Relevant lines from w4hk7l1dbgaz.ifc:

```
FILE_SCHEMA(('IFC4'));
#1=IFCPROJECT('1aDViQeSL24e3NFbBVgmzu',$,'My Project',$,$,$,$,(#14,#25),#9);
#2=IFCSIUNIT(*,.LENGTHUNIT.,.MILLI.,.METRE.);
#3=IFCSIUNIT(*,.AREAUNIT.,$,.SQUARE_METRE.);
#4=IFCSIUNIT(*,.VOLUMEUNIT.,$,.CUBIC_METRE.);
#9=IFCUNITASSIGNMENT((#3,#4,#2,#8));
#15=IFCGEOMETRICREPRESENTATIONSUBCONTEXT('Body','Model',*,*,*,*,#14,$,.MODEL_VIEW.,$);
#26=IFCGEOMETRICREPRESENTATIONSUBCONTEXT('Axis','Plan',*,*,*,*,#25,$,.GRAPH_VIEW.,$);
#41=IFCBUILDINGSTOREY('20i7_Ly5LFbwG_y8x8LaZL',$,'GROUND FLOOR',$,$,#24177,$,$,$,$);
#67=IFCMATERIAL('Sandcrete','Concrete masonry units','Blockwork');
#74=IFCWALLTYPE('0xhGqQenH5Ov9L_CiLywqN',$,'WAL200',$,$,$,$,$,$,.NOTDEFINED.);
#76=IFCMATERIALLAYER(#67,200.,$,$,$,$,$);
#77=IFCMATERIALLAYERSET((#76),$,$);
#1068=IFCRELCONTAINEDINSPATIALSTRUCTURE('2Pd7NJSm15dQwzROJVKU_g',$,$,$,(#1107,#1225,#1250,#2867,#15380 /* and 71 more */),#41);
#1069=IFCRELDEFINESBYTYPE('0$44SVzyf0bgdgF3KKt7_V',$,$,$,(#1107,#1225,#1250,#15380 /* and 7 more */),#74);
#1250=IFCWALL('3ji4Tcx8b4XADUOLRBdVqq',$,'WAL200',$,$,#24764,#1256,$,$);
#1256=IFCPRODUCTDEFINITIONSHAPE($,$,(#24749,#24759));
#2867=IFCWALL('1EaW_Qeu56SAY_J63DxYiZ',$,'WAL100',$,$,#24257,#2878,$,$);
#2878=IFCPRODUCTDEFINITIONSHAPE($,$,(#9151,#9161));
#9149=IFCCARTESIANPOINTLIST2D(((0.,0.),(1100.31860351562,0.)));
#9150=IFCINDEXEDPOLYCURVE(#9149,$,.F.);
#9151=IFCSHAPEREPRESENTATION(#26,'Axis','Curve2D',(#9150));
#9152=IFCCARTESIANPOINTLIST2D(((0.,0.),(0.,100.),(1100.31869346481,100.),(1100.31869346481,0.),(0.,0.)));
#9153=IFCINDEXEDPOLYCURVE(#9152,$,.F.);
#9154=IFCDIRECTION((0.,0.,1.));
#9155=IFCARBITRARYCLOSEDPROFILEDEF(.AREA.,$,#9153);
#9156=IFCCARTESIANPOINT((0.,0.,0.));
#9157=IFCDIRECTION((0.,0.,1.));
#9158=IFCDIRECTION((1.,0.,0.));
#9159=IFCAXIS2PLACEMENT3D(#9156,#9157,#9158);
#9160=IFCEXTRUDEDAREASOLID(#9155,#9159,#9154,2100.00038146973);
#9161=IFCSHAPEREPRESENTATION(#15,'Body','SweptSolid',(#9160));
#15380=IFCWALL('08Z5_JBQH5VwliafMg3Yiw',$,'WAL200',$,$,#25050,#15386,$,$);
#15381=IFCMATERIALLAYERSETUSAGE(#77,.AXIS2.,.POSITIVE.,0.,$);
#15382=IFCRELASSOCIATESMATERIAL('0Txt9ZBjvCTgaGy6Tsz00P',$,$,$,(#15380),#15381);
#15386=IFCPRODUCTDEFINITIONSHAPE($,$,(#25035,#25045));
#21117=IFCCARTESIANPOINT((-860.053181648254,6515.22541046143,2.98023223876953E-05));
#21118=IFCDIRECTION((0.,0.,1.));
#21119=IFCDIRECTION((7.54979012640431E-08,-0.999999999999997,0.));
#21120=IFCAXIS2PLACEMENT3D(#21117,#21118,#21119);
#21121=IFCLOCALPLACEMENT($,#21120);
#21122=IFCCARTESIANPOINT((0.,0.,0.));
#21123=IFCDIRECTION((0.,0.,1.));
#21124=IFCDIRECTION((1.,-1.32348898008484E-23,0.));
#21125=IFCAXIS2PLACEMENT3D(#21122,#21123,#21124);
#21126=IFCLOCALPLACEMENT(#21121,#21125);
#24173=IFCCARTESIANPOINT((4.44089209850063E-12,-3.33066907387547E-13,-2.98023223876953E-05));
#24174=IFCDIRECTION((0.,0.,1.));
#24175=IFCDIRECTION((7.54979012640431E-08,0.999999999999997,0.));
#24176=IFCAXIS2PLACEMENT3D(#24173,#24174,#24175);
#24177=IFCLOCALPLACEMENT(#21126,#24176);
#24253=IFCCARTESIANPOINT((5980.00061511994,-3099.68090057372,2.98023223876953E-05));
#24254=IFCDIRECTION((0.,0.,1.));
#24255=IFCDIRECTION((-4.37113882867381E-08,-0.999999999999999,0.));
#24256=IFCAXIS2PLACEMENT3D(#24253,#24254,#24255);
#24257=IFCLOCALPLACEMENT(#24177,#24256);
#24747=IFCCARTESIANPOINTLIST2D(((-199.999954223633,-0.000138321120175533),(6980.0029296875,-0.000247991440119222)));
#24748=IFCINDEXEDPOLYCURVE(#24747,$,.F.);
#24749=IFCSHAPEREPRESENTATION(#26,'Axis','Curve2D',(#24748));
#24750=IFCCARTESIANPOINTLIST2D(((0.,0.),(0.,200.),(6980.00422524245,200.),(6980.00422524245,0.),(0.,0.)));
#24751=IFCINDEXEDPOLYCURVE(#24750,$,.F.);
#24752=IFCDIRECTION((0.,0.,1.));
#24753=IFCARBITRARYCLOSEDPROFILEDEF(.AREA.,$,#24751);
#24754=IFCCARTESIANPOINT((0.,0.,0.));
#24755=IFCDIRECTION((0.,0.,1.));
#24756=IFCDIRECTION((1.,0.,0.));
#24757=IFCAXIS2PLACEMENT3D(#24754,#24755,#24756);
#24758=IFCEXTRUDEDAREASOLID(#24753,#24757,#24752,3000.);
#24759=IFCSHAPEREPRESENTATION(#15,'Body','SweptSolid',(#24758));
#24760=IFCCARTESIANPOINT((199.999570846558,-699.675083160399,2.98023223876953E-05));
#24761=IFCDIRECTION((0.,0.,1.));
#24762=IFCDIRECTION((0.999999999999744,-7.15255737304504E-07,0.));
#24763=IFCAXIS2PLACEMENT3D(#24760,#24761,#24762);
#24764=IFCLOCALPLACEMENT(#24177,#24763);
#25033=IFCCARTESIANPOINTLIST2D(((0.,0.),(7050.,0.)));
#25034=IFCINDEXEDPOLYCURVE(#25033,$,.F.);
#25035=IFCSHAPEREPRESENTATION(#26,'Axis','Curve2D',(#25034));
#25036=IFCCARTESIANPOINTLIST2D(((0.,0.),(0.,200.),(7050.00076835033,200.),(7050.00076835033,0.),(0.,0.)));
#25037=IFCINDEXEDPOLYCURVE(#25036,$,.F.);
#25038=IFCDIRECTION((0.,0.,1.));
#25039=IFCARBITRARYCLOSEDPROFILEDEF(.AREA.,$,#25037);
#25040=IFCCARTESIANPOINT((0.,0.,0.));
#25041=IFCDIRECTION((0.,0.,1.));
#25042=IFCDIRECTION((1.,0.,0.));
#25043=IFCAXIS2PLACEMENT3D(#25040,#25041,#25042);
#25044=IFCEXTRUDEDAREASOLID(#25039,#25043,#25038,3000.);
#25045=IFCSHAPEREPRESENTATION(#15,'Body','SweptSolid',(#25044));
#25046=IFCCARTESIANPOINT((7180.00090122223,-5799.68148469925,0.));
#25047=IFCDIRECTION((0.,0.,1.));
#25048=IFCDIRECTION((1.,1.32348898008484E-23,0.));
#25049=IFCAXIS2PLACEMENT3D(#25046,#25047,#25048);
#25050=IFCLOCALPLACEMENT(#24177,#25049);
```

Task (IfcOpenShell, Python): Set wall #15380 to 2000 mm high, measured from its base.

```python
import ifcopenshell
import ifcopenshell.geom
import ifcopenshell.util.representation
import ifcopenshell.util.shape
import ifcopenshell.util.unit

model = ifcopenshell.open("w4hk7l1dbgaz.ifc")
unit_scale = ifcopenshell.util.unit.calculate_unit_scale(model)
settings = ifcopenshell.geom.settings()


def volume(element):
    """Net volume in cubic metres, openings subtracted."""
    shape = ifcopenshell.geom.create_shape(settings, element)
    return ifcopenshell.util.shape.get_volume(shape.geometry)


wall = model.by_id(15380)
before = volume(wall)

body = ifcopenshell.util.representation.get_representation(wall, "Model", "Body")
solid = body.Items[0]
old_height = solid.Depth
solid.Depth = 2 / unit_scale
after = volume(wall)

print(f"height {old_height:g} -> {solid.Depth:g}, volume {before:.3f} -> {after:.3f} m3")

model.write("w4hk7l1dbgaz_v2.ifc")
```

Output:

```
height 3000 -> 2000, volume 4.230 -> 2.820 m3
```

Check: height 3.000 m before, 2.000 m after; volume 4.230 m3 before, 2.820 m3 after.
